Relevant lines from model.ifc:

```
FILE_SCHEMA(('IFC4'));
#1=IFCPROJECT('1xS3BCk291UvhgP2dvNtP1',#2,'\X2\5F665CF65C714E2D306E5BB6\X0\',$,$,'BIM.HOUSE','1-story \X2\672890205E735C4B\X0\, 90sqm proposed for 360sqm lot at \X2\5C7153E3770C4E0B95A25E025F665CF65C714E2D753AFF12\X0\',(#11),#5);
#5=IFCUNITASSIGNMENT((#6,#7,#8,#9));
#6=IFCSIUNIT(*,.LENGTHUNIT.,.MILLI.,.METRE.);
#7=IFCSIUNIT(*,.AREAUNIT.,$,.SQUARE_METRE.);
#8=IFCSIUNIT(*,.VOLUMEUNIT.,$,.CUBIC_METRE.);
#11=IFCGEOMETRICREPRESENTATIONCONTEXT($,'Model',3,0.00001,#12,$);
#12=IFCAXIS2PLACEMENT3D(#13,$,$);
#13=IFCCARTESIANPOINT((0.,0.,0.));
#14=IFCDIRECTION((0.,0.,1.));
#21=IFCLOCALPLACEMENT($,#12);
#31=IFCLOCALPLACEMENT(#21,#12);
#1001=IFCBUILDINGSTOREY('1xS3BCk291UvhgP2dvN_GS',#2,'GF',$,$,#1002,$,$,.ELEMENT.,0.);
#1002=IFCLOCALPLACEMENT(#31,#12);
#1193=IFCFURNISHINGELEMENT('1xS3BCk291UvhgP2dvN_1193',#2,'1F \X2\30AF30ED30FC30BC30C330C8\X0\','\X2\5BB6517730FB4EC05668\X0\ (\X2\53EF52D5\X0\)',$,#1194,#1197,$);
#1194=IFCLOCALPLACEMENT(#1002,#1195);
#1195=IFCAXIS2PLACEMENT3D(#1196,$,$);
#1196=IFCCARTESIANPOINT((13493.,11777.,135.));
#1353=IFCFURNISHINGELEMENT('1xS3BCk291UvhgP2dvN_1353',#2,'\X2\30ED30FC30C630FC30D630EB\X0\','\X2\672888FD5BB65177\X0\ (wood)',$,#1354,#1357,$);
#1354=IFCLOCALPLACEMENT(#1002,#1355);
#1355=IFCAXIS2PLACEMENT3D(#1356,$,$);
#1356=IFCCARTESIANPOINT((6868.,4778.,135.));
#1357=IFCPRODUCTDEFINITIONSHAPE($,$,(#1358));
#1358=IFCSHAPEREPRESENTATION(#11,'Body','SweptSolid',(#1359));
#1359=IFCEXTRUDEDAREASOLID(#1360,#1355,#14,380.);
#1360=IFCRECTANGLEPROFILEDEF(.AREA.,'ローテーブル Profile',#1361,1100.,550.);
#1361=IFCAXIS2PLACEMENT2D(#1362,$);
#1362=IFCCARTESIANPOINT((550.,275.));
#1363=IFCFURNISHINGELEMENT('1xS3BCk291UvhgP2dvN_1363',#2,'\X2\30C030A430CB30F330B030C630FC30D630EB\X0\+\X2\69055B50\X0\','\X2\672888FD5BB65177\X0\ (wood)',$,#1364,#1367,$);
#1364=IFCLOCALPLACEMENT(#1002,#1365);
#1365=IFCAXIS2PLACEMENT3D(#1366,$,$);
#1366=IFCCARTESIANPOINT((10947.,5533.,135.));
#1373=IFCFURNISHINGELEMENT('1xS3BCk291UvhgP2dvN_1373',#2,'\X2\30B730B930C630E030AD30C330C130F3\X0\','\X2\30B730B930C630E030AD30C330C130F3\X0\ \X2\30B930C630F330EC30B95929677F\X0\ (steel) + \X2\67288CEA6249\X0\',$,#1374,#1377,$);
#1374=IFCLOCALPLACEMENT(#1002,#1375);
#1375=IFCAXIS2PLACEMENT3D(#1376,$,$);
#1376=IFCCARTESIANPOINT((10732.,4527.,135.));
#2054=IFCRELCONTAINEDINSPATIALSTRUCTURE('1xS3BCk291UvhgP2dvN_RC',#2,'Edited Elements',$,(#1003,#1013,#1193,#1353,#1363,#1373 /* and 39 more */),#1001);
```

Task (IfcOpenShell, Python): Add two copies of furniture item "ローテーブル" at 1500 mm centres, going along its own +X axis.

```python
import ifcopenshell
import ifcopenshell.api.geometry
import ifcopenshell.api.root
import ifcopenshell.util.element
import ifcopenshell.util.placement
import ifcopenshell.util.unit

model = ifcopenshell.open("model.ifc")
unit_scale = ifcopenshell.util.unit.calculate_unit_scale(model)


def reuse_history(source, copy):
    """copy_class also copies each property set's owner history, people and application; keep the originals."""
    for rel in copy.IsDefinedBy:
        if rel.is_a("IfcRelDefinesByProperties") and (history := rel.RelatingPropertyDefinition.OwnerHistory):
            rel.RelatingPropertyDefinition.OwnerHistory = source.OwnerHistory
            ifcopenshell.util.element.remove_deep2(model, history)


source = model.by_guid("1xS3BCk291UvhgP2dvN_1353")
base = ifcopenshell.util.placement.get_local_placement(source.ObjectPlacement)
step = base[:3, 0] * 1.5 / unit_scale

for i in range(1, 3):
    copy = ifcopenshell.api.root.copy_class(model, product=source)
    copy.Representation = ifcopenshell.util.element.copy_deep(
        model, source.Representation, exclude=["IfcGeometricRepresentationContext", "IfcRepresentationMap"]
    )
    reuse_history(source, copy)
    matrix = base.copy()
    matrix[:3, 3] += i * step
    print("added at", matrix[:3, 3].round(3) + 0.0)
    ifcopenshell.api.geometry.edit_object_placement(model, product=copy, matrix=matrix, is_si=False)

model.write("model_rev.ifc")
```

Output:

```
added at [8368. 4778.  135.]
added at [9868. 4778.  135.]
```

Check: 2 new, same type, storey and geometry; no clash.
